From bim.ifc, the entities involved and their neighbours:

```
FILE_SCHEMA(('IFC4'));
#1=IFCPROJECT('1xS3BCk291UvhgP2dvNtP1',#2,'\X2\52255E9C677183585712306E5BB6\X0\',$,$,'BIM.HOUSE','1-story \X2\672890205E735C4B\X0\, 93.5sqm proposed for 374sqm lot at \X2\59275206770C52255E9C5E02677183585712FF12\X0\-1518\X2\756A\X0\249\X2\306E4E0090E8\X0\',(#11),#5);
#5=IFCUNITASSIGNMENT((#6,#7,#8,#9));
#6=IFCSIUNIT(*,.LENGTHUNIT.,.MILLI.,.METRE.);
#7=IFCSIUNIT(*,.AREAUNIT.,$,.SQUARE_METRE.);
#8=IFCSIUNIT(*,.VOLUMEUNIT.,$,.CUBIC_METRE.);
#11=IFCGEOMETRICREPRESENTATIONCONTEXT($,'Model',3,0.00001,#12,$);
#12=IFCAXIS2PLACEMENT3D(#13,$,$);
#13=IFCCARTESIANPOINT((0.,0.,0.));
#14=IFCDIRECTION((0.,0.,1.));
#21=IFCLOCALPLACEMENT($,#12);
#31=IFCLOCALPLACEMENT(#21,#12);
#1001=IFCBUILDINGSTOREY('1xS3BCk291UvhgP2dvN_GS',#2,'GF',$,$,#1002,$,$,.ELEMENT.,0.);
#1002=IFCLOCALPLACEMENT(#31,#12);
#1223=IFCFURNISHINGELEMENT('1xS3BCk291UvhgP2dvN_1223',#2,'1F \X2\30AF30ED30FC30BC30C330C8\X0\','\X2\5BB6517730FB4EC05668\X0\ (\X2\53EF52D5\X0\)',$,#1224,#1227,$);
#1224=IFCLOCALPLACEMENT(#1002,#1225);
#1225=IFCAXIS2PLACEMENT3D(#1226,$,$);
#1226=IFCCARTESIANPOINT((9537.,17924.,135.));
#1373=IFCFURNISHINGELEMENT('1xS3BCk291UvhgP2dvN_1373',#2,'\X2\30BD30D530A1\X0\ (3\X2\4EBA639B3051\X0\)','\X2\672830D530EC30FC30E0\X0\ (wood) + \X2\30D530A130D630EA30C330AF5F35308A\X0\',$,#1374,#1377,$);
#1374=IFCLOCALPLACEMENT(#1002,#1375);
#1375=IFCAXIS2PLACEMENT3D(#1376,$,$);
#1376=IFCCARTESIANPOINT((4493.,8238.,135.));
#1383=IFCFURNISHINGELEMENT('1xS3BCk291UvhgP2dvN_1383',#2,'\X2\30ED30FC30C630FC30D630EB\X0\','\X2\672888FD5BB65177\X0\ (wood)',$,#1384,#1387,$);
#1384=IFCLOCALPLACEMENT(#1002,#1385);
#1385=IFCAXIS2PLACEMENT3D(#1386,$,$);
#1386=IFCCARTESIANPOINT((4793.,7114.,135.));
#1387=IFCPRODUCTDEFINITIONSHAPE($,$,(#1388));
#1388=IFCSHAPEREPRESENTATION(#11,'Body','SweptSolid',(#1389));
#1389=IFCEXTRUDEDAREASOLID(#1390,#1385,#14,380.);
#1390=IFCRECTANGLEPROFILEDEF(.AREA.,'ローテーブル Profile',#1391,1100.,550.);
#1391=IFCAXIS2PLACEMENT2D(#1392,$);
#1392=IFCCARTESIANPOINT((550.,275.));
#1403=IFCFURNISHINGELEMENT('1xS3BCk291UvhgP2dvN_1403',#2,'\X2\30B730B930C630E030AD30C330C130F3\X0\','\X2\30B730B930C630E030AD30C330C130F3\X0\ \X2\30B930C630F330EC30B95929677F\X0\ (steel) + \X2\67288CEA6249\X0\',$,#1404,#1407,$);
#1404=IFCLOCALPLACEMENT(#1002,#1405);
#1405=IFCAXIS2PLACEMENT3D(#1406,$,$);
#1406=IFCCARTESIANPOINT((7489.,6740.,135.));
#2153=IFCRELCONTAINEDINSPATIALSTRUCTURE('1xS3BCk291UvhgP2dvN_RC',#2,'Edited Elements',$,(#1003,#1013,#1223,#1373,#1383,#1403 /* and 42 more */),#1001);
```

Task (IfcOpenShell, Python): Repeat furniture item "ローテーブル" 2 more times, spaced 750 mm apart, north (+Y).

```python
import numpy as np
import ifcopenshell
import ifcopenshell.api.geometry
import ifcopenshell.api.root
import ifcopenshell.util.element
import ifcopenshell.util.placement

model = ifcopenshell.open("bim.ifc")


def reuse_history(source, copy):
    """copy_class also copies each property set's owner history, people and application; keep the originals."""
    for rel in copy.IsDefinedBy:
        if rel.is_a("IfcRelDefinesByProperties") and (history := rel.RelatingPropertyDefinition.OwnerHistory):
            rel.RelatingPropertyDefinition.OwnerHistory = source.OwnerHistory
            ifcopenshell.util.element.remove_deep2(model, history)


source = model.by_guid("1xS3BCk291UvhgP2dvN_1383")
base = ifcopenshell.util.placement.get_local_placement(source.ObjectPlacement)
step = np.array([0.0, 1.0, 0.0]) * 750.0

for i in range(1, 3):
    copy = ifcopenshell.api.root.copy_class(model, product=source)
    copy.Representation = ifcopenshell.util.element.copy_deep(
        model, source.Representation, exclude=["IfcGeometricRepresentationContext", "IfcRepresentationMap"]
    )
    reuse_history(source, copy)
    matrix = base.copy()
    matrix[:3, 3] += i * step
    print("added at", matrix[:3, 3].round(3) + 0.0)
    ifcopenshell.api.geometry.edit_object_placement(model, product=copy, matrix=matrix, is_si=False)

model.write("bim_edited.ifc")
```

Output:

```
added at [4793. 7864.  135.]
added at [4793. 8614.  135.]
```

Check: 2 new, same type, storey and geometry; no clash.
